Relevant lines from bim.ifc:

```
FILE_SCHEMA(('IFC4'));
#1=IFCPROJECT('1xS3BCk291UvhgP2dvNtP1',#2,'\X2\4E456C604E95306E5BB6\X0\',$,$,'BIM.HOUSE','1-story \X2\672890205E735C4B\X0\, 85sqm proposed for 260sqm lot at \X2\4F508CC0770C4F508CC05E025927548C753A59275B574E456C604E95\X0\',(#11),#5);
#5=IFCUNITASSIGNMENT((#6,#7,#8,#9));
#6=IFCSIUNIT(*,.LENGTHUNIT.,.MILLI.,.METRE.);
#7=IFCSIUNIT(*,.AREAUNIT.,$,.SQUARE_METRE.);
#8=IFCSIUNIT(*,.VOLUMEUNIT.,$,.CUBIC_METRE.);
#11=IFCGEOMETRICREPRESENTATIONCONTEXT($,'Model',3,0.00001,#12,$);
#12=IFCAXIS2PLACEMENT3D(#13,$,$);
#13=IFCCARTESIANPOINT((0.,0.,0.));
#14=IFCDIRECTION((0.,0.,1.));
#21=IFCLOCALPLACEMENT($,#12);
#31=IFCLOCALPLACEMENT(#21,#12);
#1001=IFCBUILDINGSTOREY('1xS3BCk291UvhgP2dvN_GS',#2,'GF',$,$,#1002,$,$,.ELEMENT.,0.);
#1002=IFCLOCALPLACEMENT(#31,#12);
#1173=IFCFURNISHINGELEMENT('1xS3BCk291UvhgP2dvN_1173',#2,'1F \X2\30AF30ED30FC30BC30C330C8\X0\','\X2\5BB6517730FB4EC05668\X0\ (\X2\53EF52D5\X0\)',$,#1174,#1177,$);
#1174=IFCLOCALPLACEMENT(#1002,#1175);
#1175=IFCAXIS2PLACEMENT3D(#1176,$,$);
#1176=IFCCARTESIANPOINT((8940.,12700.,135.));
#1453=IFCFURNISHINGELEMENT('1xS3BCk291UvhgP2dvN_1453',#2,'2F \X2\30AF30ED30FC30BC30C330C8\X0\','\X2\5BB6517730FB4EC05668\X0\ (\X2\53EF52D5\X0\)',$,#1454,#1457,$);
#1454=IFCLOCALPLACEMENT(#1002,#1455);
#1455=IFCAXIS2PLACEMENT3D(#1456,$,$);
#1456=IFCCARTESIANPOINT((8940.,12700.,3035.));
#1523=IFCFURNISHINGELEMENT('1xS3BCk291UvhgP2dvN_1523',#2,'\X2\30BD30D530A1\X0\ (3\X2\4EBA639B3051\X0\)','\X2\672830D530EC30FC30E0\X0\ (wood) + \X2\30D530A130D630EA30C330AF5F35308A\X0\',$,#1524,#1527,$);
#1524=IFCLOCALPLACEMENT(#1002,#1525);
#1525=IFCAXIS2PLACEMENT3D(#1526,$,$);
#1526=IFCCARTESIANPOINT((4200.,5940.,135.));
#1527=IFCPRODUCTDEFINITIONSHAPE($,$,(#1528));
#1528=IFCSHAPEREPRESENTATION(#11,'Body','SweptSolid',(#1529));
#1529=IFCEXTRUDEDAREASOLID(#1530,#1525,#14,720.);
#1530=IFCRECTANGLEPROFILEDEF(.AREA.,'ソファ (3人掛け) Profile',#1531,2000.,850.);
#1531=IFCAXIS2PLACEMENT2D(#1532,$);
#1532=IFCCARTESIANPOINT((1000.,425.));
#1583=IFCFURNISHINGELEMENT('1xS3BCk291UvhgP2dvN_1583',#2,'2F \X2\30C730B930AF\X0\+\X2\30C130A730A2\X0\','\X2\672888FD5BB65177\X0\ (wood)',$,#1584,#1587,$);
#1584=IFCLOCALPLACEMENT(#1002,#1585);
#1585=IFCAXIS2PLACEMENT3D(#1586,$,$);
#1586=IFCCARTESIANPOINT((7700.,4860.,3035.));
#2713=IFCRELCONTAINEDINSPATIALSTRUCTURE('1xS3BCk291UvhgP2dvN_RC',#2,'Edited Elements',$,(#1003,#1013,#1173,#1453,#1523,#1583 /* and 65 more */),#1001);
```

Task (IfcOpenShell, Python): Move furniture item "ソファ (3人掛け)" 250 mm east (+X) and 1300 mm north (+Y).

```python
import ifcopenshell
import ifcopenshell.api.geometry
import ifcopenshell.util.placement

model = ifcopenshell.open("bim.ifc")

item = model.by_guid("1xS3BCk291UvhgP2dvN_1523")
matrix = ifcopenshell.util.placement.get_local_placement(item.ObjectPlacement)
matrix[0, 3] += 250.0
matrix[1, 3] += 1300.0
ifcopenshell.api.geometry.edit_object_placement(model, product=item, matrix=matrix, is_si=False)

print(ifcopenshell.util.placement.get_local_placement(item.ObjectPlacement).round(3) + 0.0)

model.write("bim_rev.ifc")
```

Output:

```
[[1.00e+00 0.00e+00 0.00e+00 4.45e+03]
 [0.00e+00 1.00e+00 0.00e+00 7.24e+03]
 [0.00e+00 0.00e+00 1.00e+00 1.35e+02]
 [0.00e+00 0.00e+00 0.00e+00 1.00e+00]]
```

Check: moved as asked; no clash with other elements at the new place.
